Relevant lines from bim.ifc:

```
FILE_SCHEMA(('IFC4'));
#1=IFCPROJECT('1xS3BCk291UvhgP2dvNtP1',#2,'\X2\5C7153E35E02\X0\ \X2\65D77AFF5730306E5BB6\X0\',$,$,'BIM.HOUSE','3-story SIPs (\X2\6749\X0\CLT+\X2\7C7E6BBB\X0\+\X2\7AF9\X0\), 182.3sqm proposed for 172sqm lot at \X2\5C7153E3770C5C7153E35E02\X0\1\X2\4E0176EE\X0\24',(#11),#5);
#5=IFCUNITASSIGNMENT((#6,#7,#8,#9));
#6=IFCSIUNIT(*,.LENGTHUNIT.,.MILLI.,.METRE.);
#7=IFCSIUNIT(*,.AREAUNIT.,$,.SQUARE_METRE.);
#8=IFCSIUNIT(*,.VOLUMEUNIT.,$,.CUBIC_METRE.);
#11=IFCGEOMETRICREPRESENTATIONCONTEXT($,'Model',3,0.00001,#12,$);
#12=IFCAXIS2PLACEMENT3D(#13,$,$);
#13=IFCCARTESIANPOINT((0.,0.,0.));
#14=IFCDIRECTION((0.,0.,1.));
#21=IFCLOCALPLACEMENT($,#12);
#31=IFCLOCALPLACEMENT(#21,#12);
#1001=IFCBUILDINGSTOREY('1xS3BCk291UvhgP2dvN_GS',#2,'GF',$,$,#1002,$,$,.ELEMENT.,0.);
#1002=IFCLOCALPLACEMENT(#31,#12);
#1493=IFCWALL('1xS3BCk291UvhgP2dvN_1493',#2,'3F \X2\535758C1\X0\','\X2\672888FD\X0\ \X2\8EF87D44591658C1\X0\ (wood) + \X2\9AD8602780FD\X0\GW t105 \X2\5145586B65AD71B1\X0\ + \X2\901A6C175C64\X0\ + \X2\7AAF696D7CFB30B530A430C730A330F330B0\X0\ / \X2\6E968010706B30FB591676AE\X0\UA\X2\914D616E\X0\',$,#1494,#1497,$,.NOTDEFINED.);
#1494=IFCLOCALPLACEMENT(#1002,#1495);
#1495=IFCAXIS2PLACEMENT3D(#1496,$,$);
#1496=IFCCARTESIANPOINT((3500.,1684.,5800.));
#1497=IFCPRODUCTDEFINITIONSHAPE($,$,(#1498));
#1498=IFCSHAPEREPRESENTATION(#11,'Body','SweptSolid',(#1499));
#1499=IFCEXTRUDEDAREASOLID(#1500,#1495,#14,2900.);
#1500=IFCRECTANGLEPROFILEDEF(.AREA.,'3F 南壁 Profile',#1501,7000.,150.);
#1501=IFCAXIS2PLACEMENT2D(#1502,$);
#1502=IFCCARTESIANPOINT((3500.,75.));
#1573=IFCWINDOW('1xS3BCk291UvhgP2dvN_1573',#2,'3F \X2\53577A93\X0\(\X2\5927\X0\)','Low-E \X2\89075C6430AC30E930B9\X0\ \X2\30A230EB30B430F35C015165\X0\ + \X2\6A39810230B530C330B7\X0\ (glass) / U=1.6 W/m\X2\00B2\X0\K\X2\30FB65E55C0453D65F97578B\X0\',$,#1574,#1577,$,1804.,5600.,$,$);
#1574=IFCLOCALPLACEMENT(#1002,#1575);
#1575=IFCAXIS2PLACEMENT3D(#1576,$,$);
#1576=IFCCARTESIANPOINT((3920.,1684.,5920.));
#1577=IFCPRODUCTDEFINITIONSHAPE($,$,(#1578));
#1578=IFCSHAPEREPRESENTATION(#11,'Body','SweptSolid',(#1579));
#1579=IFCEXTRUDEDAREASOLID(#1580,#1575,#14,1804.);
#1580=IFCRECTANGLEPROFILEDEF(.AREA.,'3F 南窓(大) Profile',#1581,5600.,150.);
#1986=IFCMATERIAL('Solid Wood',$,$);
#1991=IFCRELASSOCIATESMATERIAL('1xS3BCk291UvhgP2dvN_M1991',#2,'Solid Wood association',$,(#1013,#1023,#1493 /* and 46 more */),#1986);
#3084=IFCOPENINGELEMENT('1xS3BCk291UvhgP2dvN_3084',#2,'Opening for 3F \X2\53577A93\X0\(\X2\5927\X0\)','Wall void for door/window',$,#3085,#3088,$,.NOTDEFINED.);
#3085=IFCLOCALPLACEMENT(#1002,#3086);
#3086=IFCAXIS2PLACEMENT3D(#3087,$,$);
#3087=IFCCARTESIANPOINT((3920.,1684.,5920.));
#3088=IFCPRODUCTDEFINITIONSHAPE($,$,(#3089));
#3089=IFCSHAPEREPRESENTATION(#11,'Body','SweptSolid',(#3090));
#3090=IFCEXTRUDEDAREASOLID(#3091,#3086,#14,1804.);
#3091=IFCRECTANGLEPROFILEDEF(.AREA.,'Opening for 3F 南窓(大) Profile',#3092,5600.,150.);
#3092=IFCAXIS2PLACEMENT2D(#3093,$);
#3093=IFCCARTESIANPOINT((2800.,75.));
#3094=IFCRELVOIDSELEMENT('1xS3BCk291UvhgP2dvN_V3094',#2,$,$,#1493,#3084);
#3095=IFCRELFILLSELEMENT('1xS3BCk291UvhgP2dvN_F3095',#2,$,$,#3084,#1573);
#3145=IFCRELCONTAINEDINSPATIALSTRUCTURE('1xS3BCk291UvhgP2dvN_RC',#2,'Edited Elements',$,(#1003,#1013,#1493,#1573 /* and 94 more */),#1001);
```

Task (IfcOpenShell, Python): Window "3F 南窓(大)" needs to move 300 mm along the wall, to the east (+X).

```python
import ifcopenshell
import ifcopenshell.api.geometry
import ifcopenshell.util.placement
import ifcopenshell.util.unit

model = ifcopenshell.open("bim.ifc")
unit_scale = ifcopenshell.util.unit.calculate_unit_scale(model)

window = model.by_guid("1xS3BCk291UvhgP2dvN_1573")
opening = window.FillsVoids[0].RelatingOpeningElement
wall = opening.VoidsElements[0].RelatingBuildingElement

wall_matrix = ifcopenshell.util.placement.get_local_placement(wall.ObjectPlacement)
shift = wall_matrix[:3, 0] * 0.3 / unit_scale
before = ifcopenshell.util.placement.get_local_placement(window.ObjectPlacement)[:3, 3].copy()

# The window is not placed relative to its opening, so move both.
for product in (opening, window):
    matrix = ifcopenshell.util.placement.get_local_placement(product.ObjectPlacement)
    matrix[:3, 3] += shift
    ifcopenshell.api.geometry.edit_object_placement(model, product=product, matrix=matrix, is_si=False)

after = ifcopenshell.util.placement.get_local_placement(window.ObjectPlacement)[:3, 3]
print("window moved by", (after - before).round(3) + 0.0)

model.write("bim_edited.ifc")
```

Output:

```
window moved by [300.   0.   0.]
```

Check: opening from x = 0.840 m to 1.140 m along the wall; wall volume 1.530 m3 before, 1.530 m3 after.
